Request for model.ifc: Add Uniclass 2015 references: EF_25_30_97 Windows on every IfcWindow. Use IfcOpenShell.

First a look at what the model holds.

```python
import ifcopenshell

model = ifcopenshell.open("model.ifc")
print(model.schema)
print("classifications:", [c.Name for c in model.by_type("IfcClassification")])
for ifc_class in ("IfcDoor", "IfcRoof", "IfcStair", "IfcWall", "IfcWindow"):
    print(ifc_class, len(model.by_type(ifc_class)))
```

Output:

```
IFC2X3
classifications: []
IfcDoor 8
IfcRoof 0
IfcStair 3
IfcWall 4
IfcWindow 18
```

```python
import ifcopenshell
import ifcopenshell.api.classification

model = ifcopenshell.open("model.ifc")

# IFC2X3 requires Source and Edition and has no link from the project to the system.
system = model.create_entity("IfcClassification", Source="NBS", Edition="2015", Name="Uniclass 2015")

codes = {
    "IfcWindow": ("EF_25_30_97", "Windows"),
}
for ifc_class, (code, name) in codes.items():
    products = model.by_type(ifc_class)
    ifcopenshell.api.classification.add_reference(
        model, products=products, classification=system, identification=code, name=name
    )
    print(code, len(products))

model.write("model_updated.ifc")
```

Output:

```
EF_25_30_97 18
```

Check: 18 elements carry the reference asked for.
